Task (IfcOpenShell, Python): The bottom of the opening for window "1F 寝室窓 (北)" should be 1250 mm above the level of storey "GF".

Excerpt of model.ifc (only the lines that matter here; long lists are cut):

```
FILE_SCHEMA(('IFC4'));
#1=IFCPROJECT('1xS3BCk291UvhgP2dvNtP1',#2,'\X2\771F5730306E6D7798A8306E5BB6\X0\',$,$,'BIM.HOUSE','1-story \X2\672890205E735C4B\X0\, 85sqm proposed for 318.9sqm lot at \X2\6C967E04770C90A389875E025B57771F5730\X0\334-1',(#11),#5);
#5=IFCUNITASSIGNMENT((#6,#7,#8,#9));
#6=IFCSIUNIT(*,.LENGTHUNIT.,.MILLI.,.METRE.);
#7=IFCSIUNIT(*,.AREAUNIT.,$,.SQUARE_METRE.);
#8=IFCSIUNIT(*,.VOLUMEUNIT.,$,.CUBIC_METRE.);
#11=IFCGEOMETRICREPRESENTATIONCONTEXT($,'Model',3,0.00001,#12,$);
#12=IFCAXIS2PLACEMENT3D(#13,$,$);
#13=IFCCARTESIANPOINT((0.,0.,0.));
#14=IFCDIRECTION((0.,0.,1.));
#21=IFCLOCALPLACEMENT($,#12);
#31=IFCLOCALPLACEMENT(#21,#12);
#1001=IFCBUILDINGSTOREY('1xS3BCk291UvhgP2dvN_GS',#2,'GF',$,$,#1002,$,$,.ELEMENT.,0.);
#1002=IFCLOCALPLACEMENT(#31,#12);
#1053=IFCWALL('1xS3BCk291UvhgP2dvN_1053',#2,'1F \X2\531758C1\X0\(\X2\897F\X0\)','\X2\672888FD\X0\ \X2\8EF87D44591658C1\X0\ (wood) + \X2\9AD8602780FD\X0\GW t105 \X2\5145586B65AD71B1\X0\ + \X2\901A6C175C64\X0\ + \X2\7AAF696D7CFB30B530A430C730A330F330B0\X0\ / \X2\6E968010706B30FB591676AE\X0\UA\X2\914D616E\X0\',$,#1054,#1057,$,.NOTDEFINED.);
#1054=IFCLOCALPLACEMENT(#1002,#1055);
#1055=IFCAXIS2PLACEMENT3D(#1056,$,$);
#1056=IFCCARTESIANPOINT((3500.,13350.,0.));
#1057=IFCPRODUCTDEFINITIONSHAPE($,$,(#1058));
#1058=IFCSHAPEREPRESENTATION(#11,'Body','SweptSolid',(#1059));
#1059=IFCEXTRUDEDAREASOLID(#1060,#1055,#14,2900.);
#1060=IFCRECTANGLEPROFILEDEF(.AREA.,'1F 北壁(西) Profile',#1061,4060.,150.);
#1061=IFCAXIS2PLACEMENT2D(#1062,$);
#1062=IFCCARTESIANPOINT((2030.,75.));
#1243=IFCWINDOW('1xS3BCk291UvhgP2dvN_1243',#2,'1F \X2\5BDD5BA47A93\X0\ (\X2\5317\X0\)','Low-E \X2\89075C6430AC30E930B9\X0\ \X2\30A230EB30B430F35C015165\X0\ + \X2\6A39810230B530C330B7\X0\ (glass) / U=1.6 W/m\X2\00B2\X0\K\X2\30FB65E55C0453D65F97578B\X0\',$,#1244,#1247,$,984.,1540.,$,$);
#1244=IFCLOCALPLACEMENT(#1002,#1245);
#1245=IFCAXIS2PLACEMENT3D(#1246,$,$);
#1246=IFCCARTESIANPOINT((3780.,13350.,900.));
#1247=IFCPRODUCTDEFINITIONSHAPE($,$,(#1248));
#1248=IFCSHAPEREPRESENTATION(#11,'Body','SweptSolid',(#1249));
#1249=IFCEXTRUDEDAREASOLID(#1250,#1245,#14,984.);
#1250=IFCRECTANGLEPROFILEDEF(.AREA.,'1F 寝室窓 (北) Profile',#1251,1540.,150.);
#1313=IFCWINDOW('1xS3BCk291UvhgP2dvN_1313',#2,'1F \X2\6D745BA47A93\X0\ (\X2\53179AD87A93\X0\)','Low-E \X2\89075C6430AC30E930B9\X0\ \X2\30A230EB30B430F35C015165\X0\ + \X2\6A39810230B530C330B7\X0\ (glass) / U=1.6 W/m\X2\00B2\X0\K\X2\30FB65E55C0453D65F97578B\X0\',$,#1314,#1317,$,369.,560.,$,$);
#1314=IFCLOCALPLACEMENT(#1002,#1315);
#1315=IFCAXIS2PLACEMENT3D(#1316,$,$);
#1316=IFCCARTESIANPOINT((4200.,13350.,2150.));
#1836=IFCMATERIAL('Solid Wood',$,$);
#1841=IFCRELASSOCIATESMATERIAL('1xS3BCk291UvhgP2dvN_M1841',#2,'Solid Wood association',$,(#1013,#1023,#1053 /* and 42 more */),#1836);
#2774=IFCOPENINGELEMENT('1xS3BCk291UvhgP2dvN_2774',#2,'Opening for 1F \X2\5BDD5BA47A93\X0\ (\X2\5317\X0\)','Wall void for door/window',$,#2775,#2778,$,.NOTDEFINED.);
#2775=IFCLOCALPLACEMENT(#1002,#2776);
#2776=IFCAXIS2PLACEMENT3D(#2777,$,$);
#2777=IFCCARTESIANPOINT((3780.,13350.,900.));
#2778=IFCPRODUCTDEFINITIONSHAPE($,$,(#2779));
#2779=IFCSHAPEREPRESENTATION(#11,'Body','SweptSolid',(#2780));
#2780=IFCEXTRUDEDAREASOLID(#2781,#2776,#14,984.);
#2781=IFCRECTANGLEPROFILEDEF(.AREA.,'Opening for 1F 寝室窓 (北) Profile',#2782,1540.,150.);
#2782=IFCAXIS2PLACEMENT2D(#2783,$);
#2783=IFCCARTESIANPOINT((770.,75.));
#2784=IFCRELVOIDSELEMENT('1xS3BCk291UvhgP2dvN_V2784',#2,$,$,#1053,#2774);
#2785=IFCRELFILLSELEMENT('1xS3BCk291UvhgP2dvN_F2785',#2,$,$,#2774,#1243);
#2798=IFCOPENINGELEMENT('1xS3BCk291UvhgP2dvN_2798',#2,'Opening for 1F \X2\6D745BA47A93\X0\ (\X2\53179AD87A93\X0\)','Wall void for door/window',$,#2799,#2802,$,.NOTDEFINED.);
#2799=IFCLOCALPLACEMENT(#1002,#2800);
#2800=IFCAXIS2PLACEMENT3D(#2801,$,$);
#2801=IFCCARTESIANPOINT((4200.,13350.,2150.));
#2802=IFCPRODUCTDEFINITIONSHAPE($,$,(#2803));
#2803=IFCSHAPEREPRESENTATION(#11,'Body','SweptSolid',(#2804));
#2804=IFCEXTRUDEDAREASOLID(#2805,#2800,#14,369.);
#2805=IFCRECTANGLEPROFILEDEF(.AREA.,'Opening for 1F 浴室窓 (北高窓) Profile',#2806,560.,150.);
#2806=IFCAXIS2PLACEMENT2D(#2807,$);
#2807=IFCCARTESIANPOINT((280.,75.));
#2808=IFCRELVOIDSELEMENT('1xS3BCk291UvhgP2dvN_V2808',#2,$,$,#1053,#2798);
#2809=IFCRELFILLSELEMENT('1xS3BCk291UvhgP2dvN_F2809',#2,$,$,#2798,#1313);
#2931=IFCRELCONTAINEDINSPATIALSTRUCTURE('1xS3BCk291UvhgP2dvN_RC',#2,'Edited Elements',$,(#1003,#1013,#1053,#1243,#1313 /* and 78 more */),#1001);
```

```python
import numpy as np
import ifcopenshell
import ifcopenshell.api.geometry
import ifcopenshell.geom
import ifcopenshell.util.element
import ifcopenshell.util.placement
import ifcopenshell.util.shape
import ifcopenshell.util.unit

model = ifcopenshell.open("model.ifc")
unit_scale = ifcopenshell.util.unit.calculate_unit_scale(model)

window = model.by_guid("1xS3BCk291UvhgP2dvN_1243")
opening = window.FillsVoids[0].RelatingOpeningElement
storey = ifcopenshell.util.element.get_container(window, ifc_class="IfcBuildingStorey")
level = ifcopenshell.util.placement.get_local_placement(storey.ObjectPlacement)[2, 3]

# The opening's origin need not be at the sill, so measure its lowest point.
shape = ifcopenshell.geom.create_shape(ifcopenshell.geom.settings(), opening)
bottom = ifcopenshell.util.shape.get_shape_bottom_elevation(shape, shape.geometry) / unit_scale
dz = level + 1250.0 - bottom

shift = np.array([0.0, 0.0, dz])
# The window is not placed relative to its opening, so move both.
for product in (opening, window):
    matrix = ifcopenshell.util.placement.get_local_placement(product.ObjectPlacement)
    matrix[:3, 3] += shift
    ifcopenshell.api.geometry.edit_object_placement(model, product=product, matrix=matrix, is_si=False)

print(f"moved by {dz * unit_scale:+.3f} m")

model.write("model_updated.ifc")
```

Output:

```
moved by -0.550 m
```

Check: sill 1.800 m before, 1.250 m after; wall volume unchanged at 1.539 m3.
